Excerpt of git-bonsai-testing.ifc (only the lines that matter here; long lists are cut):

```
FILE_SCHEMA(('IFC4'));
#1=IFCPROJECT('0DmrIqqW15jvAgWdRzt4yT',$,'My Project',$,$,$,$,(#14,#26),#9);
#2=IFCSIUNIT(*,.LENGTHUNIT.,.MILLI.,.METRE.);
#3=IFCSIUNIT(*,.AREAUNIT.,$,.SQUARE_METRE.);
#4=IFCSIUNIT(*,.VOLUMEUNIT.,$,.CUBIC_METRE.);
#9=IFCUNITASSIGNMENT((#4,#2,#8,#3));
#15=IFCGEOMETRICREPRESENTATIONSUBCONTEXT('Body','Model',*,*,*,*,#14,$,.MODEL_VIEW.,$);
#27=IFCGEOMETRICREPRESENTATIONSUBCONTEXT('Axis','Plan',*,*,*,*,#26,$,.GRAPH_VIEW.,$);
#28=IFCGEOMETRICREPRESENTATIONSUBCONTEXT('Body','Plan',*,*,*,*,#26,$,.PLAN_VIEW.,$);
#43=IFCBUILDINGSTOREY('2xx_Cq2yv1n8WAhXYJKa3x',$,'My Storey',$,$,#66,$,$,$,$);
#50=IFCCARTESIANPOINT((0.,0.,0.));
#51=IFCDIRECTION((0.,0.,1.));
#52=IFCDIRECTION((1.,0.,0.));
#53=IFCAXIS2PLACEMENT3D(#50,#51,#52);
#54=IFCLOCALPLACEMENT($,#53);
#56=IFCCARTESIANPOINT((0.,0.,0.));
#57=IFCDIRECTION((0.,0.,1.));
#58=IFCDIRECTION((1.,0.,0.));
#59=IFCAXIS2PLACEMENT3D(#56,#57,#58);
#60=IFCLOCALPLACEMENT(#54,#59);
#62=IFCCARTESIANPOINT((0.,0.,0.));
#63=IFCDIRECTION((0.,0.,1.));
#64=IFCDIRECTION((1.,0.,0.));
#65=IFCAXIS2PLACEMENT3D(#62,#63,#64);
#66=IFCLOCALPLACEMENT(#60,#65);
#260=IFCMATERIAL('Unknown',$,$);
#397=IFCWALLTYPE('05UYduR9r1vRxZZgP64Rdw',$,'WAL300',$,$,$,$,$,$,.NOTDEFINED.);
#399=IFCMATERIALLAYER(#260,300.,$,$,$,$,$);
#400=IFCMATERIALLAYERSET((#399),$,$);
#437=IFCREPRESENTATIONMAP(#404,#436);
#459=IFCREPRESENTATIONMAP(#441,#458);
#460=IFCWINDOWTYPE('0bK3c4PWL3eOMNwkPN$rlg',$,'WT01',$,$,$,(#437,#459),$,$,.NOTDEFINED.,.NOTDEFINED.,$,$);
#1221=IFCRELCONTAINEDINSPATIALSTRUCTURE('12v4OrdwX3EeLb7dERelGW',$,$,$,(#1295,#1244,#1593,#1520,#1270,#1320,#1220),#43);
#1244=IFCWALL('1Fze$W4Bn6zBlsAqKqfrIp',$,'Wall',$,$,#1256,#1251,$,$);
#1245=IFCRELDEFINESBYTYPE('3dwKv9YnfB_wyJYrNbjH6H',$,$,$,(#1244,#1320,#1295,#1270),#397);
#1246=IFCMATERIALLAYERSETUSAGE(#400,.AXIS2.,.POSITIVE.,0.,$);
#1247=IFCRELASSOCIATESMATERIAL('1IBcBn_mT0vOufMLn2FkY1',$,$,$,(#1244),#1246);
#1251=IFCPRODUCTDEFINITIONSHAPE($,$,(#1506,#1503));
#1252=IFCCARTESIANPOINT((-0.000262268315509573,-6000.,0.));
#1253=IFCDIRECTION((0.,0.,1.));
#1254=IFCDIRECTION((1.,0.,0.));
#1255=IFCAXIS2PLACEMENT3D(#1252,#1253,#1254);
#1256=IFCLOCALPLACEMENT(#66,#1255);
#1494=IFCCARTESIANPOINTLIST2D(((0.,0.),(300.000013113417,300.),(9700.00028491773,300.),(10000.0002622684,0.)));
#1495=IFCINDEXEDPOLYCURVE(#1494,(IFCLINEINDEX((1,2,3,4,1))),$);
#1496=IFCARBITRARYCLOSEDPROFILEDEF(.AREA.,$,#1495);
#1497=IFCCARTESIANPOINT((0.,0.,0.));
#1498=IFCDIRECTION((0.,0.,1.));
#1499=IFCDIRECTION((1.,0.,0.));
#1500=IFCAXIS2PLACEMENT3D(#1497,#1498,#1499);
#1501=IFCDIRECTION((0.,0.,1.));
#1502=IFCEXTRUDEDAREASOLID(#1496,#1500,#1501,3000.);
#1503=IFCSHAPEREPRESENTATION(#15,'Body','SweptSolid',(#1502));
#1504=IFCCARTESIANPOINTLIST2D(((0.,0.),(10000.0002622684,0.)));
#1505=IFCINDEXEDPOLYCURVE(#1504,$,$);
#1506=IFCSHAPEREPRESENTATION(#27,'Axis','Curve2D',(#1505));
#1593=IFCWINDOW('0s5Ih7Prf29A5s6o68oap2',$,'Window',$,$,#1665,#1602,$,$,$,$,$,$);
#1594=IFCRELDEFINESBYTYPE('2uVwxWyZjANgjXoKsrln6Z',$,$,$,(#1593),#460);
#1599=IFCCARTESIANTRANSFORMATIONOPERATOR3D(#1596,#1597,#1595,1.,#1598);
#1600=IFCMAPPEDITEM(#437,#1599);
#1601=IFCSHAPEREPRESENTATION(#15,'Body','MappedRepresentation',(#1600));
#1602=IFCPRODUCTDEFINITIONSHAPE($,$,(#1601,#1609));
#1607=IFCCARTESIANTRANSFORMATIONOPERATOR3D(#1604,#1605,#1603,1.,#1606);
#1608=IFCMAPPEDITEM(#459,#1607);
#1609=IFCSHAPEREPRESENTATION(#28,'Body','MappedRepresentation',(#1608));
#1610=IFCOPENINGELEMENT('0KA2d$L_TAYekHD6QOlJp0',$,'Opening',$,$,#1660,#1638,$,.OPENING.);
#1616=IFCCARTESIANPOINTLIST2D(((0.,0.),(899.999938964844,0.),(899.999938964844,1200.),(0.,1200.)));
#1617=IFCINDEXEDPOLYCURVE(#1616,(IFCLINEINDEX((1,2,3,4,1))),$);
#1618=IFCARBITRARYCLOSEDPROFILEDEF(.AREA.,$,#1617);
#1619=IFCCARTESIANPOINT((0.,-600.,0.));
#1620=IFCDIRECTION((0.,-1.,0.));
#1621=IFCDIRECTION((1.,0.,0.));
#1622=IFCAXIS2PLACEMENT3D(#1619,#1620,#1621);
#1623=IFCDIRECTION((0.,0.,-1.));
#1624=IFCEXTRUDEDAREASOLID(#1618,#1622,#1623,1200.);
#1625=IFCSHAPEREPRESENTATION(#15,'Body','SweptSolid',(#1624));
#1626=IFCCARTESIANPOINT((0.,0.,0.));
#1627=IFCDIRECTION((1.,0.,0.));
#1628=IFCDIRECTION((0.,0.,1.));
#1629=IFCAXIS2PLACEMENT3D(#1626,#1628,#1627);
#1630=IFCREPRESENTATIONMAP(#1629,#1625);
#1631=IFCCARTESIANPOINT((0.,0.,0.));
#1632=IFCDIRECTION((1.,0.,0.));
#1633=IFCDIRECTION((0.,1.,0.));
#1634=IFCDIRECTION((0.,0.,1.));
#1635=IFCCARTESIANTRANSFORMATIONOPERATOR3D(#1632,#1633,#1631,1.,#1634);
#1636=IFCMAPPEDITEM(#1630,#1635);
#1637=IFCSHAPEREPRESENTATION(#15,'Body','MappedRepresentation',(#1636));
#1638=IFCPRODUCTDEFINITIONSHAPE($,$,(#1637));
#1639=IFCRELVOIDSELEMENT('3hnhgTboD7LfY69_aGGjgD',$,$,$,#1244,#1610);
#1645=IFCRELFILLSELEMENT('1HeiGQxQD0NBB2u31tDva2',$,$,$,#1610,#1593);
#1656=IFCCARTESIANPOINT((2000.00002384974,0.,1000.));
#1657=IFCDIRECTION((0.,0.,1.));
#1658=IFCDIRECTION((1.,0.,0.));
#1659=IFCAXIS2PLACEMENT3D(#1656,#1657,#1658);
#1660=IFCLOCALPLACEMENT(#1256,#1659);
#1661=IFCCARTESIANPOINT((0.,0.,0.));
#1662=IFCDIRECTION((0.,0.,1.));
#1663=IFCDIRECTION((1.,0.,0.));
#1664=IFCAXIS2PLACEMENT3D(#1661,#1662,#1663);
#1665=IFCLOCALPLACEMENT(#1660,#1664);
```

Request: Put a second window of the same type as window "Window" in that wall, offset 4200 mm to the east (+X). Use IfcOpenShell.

```python
import ifcopenshell
import ifcopenshell.api.feature
import ifcopenshell.api.geometry
import ifcopenshell.api.root
import ifcopenshell.geom
import ifcopenshell.util.element
import ifcopenshell.util.placement
import ifcopenshell.util.shape

model = ifcopenshell.open("git-bonsai-testing.ifc")
settings = ifcopenshell.geom.settings()


def volume(element):
    """Net volume in cubic metres, openings subtracted."""
    shape = ifcopenshell.geom.create_shape(settings, element)
    return ifcopenshell.util.shape.get_volume(shape.geometry)


window = model.by_guid("0s5Ih7Prf29A5s6o68oap2")
opening = window.FillsVoids[0].RelatingOpeningElement
wall = opening.VoidsElements[0].RelatingBuildingElement
before = volume(wall)
shift = ifcopenshell.util.placement.get_local_placement(wall.ObjectPlacement)[:3, 0] * 4200.0

# copy_class copies the void relationship, type, container and properties, but no geometry.
new_opening = ifcopenshell.api.root.copy_class(model, product=opening)
new_opening.Representation = ifcopenshell.util.element.copy_deep(
    model, opening.Representation, exclude=["IfcGeometricRepresentationContext", "IfcRepresentationMap"]
)
new_window = ifcopenshell.api.root.copy_class(model, product=window)
new_window.Representation = ifcopenshell.util.element.copy_deep(
    model, window.Representation, exclude=["IfcGeometricRepresentationContext", "IfcRepresentationMap"]
)
ifcopenshell.api.feature.add_filling(model, opening=new_opening, element=new_window)

for old, new in ((opening, new_opening), (window, new_window)):
    matrix = ifcopenshell.util.placement.get_local_placement(old.ObjectPlacement)
    matrix[:3, 3] += shift
    ifcopenshell.api.geometry.edit_object_placement(model, product=new, matrix=matrix, is_si=False)

after = volume(wall)

print(f"wall volume {before:.3f} -> {after:.3f} m3")

model.write("git-bonsai-testing_rev.ifc")
```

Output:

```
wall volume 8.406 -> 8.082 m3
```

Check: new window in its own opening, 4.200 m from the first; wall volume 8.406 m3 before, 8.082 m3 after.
